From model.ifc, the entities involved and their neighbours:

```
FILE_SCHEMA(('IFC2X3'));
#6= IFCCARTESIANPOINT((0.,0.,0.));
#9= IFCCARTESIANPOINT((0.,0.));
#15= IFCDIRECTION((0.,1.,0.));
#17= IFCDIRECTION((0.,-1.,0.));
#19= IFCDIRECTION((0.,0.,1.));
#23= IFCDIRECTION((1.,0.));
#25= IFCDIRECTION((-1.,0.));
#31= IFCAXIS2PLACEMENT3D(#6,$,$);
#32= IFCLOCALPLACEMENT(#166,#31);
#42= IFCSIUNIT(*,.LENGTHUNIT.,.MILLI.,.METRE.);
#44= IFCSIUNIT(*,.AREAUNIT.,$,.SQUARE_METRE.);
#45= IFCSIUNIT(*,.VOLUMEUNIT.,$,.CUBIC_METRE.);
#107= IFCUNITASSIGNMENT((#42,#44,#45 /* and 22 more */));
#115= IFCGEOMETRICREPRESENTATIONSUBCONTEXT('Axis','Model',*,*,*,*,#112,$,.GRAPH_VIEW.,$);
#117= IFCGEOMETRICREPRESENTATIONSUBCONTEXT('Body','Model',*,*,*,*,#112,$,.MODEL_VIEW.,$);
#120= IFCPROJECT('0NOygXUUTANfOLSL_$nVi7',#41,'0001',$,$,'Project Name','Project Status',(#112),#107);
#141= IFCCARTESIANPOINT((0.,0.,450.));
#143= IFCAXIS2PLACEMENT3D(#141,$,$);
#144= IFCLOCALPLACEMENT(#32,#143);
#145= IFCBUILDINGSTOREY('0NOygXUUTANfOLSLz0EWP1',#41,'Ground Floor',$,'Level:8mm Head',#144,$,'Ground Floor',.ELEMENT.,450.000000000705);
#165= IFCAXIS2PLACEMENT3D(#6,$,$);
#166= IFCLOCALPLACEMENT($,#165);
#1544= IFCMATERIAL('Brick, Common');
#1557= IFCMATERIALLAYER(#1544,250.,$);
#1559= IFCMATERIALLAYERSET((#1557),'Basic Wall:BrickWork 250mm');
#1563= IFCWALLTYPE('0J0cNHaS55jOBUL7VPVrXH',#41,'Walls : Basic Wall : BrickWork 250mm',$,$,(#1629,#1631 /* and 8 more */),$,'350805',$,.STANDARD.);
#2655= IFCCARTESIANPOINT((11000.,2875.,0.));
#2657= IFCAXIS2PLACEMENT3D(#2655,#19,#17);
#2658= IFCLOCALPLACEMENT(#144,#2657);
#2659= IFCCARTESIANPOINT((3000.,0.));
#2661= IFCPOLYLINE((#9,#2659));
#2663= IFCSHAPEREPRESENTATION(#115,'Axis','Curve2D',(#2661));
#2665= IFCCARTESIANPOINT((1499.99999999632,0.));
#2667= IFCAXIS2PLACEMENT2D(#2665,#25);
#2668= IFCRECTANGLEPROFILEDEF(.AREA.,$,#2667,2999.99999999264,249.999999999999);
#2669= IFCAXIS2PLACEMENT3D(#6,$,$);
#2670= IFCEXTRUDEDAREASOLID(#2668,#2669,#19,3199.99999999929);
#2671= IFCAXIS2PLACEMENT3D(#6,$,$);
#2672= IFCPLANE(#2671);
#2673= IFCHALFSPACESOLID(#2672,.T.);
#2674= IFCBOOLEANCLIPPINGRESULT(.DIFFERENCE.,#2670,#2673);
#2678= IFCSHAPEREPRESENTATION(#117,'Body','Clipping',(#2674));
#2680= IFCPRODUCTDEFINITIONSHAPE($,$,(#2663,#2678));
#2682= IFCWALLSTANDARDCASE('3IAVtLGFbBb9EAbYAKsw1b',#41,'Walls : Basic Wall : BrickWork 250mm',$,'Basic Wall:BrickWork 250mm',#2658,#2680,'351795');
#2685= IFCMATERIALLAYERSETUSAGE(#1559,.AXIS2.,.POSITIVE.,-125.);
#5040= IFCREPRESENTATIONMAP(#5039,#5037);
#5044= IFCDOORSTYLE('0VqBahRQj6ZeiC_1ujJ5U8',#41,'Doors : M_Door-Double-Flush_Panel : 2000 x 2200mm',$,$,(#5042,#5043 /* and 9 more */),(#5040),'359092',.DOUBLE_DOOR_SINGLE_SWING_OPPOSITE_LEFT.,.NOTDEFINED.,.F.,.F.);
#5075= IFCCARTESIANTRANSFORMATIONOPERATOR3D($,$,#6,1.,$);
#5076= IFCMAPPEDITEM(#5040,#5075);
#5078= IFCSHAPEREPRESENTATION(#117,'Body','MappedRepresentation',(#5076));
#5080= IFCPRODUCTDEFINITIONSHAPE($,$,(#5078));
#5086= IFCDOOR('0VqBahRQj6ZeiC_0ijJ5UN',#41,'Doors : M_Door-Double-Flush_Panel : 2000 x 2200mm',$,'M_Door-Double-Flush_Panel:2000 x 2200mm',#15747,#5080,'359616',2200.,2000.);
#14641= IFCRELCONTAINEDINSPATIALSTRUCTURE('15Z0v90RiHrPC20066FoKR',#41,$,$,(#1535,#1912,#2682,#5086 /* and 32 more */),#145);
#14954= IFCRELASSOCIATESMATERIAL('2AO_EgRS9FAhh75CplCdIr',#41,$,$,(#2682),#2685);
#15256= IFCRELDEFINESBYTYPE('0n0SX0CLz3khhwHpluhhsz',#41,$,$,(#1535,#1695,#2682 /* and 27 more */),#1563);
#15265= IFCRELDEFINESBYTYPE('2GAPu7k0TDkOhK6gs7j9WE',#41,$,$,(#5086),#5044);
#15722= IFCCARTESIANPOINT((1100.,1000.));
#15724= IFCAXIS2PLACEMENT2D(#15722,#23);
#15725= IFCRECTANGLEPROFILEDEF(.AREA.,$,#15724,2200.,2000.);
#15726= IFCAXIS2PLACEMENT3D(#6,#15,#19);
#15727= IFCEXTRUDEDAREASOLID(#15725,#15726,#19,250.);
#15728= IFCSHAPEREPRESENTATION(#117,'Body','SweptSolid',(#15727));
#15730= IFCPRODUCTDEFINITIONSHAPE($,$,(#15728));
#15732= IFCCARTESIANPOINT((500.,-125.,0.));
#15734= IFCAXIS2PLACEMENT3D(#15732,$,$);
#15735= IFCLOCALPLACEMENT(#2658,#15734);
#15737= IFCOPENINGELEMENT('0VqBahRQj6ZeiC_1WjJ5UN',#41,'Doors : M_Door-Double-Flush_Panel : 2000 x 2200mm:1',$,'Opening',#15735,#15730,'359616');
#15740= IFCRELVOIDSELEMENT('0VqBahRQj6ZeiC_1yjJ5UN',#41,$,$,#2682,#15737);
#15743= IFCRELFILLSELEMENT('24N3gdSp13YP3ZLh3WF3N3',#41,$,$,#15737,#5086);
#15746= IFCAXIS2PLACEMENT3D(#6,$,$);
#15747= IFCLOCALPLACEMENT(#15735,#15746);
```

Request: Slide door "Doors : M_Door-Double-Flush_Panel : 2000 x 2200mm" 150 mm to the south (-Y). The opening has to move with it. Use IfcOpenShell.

```python
import ifcopenshell
import ifcopenshell.api.geometry
import ifcopenshell.util.placement
import ifcopenshell.util.unit

model = ifcopenshell.open("model.ifc")
unit_scale = ifcopenshell.util.unit.calculate_unit_scale(model)

door = model.by_guid("0VqBahRQj6ZeiC_0ijJ5UN")
opening = door.FillsVoids[0].RelatingOpeningElement
wall = opening.VoidsElements[0].RelatingBuildingElement

wall_matrix = ifcopenshell.util.placement.get_local_placement(wall.ObjectPlacement)
shift = wall_matrix[:3, 0] * 0.15 / unit_scale
before = ifcopenshell.util.placement.get_local_placement(door.ObjectPlacement)[:3, 3].copy()

# The door is placed relative to its opening, so it follows when the opening moves.
matrix = ifcopenshell.util.placement.get_local_placement(opening.ObjectPlacement)
matrix[:3, 3] += shift
ifcopenshell.api.geometry.edit_object_placement(
    model, product=opening, matrix=matrix, is_si=False, should_transform_children=True
)

after = ifcopenshell.util.placement.get_local_placement(door.ObjectPlacement)[:3, 3]
print("door moved by", (after - before).round(3) + 0.0)

model.write("model_rev.ifc")
```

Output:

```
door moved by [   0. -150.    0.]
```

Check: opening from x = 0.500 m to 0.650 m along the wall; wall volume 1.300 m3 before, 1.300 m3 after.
